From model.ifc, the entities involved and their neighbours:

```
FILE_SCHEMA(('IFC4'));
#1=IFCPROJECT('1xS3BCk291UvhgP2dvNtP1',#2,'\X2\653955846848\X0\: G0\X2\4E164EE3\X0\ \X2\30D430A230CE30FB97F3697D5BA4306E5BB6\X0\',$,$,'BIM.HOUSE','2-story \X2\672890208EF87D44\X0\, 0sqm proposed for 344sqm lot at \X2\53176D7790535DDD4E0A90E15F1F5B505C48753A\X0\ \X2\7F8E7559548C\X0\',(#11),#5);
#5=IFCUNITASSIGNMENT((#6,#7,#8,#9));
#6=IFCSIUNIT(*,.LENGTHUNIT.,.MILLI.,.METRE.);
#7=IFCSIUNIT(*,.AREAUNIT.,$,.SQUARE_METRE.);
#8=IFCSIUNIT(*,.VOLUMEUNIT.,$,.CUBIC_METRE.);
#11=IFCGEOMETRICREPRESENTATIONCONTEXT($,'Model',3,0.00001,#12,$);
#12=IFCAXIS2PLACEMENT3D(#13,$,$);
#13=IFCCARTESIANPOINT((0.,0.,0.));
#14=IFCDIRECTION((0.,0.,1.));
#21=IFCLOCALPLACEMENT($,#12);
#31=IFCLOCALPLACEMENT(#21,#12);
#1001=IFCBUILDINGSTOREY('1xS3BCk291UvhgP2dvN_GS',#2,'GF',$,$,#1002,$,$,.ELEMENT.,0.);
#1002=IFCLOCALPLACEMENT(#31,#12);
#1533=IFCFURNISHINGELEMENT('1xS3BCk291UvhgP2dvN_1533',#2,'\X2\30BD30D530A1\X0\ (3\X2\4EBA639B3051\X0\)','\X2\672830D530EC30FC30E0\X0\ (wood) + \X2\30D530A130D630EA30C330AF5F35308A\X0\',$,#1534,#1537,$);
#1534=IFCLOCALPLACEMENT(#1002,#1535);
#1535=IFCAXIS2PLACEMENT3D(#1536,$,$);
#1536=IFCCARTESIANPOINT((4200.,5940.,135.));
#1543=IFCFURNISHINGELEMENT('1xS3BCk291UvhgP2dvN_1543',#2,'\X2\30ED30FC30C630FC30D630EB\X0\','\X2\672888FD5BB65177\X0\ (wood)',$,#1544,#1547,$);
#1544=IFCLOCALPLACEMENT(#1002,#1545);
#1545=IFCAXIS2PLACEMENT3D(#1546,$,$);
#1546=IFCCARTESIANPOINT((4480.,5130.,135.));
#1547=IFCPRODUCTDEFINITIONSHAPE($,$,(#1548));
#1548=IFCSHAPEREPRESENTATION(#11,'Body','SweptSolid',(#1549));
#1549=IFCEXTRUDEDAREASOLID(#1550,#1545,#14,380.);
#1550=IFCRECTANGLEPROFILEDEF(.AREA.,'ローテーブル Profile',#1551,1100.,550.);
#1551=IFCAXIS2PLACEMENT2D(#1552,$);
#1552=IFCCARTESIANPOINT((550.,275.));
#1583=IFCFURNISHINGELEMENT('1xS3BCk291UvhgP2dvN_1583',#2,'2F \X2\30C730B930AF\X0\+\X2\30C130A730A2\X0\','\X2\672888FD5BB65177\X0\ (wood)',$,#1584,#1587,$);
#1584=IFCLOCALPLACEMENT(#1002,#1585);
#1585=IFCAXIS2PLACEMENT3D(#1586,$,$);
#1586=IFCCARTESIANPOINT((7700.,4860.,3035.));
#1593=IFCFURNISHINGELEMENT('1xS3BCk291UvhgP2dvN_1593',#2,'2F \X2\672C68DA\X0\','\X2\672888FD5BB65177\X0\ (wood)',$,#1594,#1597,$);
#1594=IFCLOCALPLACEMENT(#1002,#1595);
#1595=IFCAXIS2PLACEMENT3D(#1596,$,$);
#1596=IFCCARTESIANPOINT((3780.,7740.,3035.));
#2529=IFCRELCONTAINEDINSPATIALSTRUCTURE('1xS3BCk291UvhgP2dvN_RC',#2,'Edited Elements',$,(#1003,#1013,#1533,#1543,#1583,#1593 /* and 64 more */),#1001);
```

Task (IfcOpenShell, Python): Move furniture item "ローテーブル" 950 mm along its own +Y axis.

```python
import ifcopenshell
import ifcopenshell.api.geometry
import ifcopenshell.util.placement
import ifcopenshell.util.unit

model = ifcopenshell.open("model.ifc")
unit_scale = ifcopenshell.util.unit.calculate_unit_scale(model)

item = model.by_id(1543)
matrix = ifcopenshell.util.placement.get_local_placement(item.ObjectPlacement)
matrix[:3, 3] += matrix[:3, 1] * 0.95 / unit_scale
ifcopenshell.api.geometry.edit_object_placement(model, product=item, matrix=matrix, is_si=False)

print(ifcopenshell.util.placement.get_local_placement(item.ObjectPlacement).round(3) + 0.0)

model.write("model_rev.ifc")
```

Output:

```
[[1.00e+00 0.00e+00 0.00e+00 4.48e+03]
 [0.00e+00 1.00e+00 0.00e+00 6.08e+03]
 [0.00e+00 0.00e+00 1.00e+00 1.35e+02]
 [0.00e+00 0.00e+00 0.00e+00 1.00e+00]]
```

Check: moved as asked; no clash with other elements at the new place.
